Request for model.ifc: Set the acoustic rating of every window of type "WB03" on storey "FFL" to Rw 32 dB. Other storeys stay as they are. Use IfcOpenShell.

First a look at what the model holds.

```python
import ifcopenshell
import ifcopenshell.util.element

model = ifcopenshell.open("model.ifc")
print(model.schema)
storey = next(s for s in model.by_type("IfcBuildingStorey") if s.Name == "FFL")
windows = [e for e in ifcopenshell.util.element.get_decomposition(storey) if e.is_a("IfcWindow")]
seen = {}
for e in windows:
    element_type = ifcopenshell.util.element.get_type(e)
    key = (element_type.Name if element_type != e and element_type else None, ifcopenshell.util.element.get_pset(e, "Pset_WindowCommon", "AcousticRating"))
    seen[key] = seen.get(key, 0) + 1
for (name, value), count in sorted(seen.items(), key=str):
    print(count, "x", name, "|", value)
```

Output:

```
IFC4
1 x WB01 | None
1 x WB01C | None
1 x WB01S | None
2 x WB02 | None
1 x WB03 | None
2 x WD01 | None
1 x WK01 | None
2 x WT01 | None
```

```python
import ifcopenshell
import ifcopenshell.api.pset
import ifcopenshell.util.element

model = ifcopenshell.open("model.ifc")

storey = next(s for s in model.by_type("IfcBuildingStorey") if s.Name == "FFL")
windows = [e for e in ifcopenshell.util.element.get_decomposition(storey) if e.is_a("IfcWindow")]

count = 0
for e in windows:
    element_type = ifcopenshell.util.element.get_type(e)
    if element_type in (None, e) or element_type.Name != "WB03":
        continue
    # add_pset returns the element's existing set when there is one.
    pset = ifcopenshell.api.pset.add_pset(model, product=e, name="Pset_WindowCommon")
    ifcopenshell.api.pset.edit_pset(model, pset=pset, properties={"AcousticRating": "Rw 32 dB"})
    count += 1

print(count, "windows updated")

model.write("model_edited.ifc")
```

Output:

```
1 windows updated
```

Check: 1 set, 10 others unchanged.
